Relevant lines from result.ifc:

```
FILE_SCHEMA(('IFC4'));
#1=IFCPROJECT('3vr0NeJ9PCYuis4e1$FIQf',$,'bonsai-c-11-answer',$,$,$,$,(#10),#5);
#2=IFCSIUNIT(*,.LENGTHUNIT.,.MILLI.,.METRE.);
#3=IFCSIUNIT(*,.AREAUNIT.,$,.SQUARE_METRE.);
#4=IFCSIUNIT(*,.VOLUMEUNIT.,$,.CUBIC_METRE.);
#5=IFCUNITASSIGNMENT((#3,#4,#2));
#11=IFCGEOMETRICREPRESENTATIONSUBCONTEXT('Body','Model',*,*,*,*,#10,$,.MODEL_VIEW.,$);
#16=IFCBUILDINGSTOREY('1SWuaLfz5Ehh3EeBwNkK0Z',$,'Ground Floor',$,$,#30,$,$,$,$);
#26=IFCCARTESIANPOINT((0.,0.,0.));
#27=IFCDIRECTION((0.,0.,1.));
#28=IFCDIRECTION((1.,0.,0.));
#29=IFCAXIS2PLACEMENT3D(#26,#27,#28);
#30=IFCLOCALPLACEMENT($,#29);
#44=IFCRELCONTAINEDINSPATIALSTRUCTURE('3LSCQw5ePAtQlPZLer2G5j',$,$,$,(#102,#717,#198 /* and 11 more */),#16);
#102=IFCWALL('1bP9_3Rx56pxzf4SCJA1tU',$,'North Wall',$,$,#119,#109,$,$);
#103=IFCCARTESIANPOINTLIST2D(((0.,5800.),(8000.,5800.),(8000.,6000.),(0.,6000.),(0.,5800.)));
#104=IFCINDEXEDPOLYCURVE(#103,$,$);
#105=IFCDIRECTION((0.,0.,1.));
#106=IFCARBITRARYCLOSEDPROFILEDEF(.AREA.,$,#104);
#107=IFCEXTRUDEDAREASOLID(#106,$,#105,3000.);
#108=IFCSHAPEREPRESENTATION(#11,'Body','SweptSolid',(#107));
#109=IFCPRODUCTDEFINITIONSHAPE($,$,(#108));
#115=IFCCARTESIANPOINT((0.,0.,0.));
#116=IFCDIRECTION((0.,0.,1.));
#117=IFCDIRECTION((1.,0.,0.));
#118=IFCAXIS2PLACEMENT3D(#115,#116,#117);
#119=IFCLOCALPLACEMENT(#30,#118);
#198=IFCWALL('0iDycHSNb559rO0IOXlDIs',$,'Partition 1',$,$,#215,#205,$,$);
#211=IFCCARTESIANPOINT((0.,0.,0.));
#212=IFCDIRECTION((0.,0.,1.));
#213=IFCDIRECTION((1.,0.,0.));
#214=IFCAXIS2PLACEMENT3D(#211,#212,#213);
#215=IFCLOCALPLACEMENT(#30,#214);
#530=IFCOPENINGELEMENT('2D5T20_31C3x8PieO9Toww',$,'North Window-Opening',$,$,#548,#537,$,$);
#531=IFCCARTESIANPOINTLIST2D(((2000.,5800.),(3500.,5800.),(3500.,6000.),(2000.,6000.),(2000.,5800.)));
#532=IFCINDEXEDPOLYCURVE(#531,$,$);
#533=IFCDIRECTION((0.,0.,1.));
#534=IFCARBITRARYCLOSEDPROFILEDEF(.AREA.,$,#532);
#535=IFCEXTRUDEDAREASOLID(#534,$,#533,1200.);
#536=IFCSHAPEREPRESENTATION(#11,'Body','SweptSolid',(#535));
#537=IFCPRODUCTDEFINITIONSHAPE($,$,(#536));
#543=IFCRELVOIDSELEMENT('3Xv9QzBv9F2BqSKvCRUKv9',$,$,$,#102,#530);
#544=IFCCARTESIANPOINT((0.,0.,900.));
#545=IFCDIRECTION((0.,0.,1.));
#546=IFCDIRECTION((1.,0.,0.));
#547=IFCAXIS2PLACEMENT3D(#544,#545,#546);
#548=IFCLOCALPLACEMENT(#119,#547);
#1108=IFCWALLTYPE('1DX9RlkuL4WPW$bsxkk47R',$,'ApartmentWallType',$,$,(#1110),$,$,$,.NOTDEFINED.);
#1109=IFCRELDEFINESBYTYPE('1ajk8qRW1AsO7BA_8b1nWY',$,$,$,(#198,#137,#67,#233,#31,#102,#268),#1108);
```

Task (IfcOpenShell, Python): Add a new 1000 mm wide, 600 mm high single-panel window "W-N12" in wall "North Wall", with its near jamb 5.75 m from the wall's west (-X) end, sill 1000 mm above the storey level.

```python
import numpy as np
import ifcopenshell
import ifcopenshell.api.feature
import ifcopenshell.api.geometry
import ifcopenshell.api.root
import ifcopenshell.api.spatial
import ifcopenshell.geom
import ifcopenshell.util.element
import ifcopenshell.util.placement
import ifcopenshell.util.representation
import ifcopenshell.util.shape
import ifcopenshell.util.unit

model = ifcopenshell.open("result.ifc")
unit_scale = ifcopenshell.util.unit.calculate_unit_scale(model)
settings = ifcopenshell.geom.settings()


def volume(element):
    """Net volume in cubic metres, openings subtracted."""
    shape = ifcopenshell.geom.create_shape(settings, element)
    return ifcopenshell.util.shape.get_volume(shape.geometry)


wall = model.by_id(102)
storey = ifcopenshell.util.element.get_container(wall, ifc_class="IfcBuildingStorey")
context = ifcopenshell.util.representation.get_context(model, "Model", "Body", "MODEL_VIEW")
before = volume(wall)

width, height, from_end, sill = 1, 0.6, 5.75, 1  # metres

# The wall runs along its own X axis, and the end named is its -X end.
wall_shape = ifcopenshell.geom.create_shape(settings, wall)
x, y, z = ifcopenshell.util.shape.get_vertices(wall_shape.geometry).T
start = x.min() + from_end
face, thickness = float(y.min()), float(y.max() - y.min())
wall_matrix = ifcopenshell.util.placement.get_local_placement(wall.ObjectPlacement)
level = ifcopenshell.util.placement.get_local_placement(storey.ObjectPlacement)[2, 3]


def in_wall(x, y):
    """Placement at x, y metres in the wall's axes, at sill height."""
    matrix = wall_matrix.copy()
    matrix[:, 3] = wall_matrix @ np.array([x / unit_scale, y / unit_scale, 0.0, 1.0])
    matrix[2, 3] = level + sill / unit_scale
    return matrix


# Opening: a box that overshoots both wall faces by 50 mm.
opening = ifcopenshell.api.root.create_entity(model, ifc_class="IfcOpeningElement", predefined_type="OPENING")
box = ifcopenshell.api.geometry.add_wall_representation(
    model, context=context, length=width, height=height, thickness=thickness + 0.1
)
ifcopenshell.api.geometry.assign_representation(model, product=opening, representation=box)
ifcopenshell.api.geometry.edit_object_placement(model, product=opening, matrix=in_wall(start, face - 0.05), is_si=False)
ifcopenshell.api.feature.add_feature(model, feature=opening, element=wall)

window = ifcopenshell.api.root.create_entity(model, ifc_class="IfcWindow", name="W-N12", predefined_type="WINDOW")
window.OverallWidth, window.OverallHeight = width / unit_scale, height / unit_scale
window.PartitioningType = "SINGLE_PANEL"
body = ifcopenshell.api.geometry.add_window_representation(
    model,
    context=context,
    overall_width=window.OverallWidth,
    overall_height=window.OverallHeight,
    partition_type="SINGLE_PANEL",
)
ifcopenshell.api.geometry.assign_representation(model, product=window, representation=body)
ifcopenshell.api.spatial.assign_container(model, products=[window], relating_structure=storey)
ifcopenshell.api.feature.add_filling(model, opening=opening, element=window)

# Centre the window in the wall's thickness.
ifcopenshell.api.geometry.edit_object_placement(model, product=window, matrix=in_wall(start, face), is_si=False)
window_shape = ifcopenshell.geom.create_shape(settings, window)
depth = ifcopenshell.util.shape.get_vertices(window_shape.geometry)[:, 1]
offset = face + thickness / 2 - (depth.min() + depth.max()) / 2
ifcopenshell.api.geometry.edit_object_placement(model, product=window, matrix=in_wall(start, offset), is_si=False)

after = volume(wall)

print(f"wall volume {before:.3f} -> {after:.3f} m3")

model.write("result_v2.ifc")
```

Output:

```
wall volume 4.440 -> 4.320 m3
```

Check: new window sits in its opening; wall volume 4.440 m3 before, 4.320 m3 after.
